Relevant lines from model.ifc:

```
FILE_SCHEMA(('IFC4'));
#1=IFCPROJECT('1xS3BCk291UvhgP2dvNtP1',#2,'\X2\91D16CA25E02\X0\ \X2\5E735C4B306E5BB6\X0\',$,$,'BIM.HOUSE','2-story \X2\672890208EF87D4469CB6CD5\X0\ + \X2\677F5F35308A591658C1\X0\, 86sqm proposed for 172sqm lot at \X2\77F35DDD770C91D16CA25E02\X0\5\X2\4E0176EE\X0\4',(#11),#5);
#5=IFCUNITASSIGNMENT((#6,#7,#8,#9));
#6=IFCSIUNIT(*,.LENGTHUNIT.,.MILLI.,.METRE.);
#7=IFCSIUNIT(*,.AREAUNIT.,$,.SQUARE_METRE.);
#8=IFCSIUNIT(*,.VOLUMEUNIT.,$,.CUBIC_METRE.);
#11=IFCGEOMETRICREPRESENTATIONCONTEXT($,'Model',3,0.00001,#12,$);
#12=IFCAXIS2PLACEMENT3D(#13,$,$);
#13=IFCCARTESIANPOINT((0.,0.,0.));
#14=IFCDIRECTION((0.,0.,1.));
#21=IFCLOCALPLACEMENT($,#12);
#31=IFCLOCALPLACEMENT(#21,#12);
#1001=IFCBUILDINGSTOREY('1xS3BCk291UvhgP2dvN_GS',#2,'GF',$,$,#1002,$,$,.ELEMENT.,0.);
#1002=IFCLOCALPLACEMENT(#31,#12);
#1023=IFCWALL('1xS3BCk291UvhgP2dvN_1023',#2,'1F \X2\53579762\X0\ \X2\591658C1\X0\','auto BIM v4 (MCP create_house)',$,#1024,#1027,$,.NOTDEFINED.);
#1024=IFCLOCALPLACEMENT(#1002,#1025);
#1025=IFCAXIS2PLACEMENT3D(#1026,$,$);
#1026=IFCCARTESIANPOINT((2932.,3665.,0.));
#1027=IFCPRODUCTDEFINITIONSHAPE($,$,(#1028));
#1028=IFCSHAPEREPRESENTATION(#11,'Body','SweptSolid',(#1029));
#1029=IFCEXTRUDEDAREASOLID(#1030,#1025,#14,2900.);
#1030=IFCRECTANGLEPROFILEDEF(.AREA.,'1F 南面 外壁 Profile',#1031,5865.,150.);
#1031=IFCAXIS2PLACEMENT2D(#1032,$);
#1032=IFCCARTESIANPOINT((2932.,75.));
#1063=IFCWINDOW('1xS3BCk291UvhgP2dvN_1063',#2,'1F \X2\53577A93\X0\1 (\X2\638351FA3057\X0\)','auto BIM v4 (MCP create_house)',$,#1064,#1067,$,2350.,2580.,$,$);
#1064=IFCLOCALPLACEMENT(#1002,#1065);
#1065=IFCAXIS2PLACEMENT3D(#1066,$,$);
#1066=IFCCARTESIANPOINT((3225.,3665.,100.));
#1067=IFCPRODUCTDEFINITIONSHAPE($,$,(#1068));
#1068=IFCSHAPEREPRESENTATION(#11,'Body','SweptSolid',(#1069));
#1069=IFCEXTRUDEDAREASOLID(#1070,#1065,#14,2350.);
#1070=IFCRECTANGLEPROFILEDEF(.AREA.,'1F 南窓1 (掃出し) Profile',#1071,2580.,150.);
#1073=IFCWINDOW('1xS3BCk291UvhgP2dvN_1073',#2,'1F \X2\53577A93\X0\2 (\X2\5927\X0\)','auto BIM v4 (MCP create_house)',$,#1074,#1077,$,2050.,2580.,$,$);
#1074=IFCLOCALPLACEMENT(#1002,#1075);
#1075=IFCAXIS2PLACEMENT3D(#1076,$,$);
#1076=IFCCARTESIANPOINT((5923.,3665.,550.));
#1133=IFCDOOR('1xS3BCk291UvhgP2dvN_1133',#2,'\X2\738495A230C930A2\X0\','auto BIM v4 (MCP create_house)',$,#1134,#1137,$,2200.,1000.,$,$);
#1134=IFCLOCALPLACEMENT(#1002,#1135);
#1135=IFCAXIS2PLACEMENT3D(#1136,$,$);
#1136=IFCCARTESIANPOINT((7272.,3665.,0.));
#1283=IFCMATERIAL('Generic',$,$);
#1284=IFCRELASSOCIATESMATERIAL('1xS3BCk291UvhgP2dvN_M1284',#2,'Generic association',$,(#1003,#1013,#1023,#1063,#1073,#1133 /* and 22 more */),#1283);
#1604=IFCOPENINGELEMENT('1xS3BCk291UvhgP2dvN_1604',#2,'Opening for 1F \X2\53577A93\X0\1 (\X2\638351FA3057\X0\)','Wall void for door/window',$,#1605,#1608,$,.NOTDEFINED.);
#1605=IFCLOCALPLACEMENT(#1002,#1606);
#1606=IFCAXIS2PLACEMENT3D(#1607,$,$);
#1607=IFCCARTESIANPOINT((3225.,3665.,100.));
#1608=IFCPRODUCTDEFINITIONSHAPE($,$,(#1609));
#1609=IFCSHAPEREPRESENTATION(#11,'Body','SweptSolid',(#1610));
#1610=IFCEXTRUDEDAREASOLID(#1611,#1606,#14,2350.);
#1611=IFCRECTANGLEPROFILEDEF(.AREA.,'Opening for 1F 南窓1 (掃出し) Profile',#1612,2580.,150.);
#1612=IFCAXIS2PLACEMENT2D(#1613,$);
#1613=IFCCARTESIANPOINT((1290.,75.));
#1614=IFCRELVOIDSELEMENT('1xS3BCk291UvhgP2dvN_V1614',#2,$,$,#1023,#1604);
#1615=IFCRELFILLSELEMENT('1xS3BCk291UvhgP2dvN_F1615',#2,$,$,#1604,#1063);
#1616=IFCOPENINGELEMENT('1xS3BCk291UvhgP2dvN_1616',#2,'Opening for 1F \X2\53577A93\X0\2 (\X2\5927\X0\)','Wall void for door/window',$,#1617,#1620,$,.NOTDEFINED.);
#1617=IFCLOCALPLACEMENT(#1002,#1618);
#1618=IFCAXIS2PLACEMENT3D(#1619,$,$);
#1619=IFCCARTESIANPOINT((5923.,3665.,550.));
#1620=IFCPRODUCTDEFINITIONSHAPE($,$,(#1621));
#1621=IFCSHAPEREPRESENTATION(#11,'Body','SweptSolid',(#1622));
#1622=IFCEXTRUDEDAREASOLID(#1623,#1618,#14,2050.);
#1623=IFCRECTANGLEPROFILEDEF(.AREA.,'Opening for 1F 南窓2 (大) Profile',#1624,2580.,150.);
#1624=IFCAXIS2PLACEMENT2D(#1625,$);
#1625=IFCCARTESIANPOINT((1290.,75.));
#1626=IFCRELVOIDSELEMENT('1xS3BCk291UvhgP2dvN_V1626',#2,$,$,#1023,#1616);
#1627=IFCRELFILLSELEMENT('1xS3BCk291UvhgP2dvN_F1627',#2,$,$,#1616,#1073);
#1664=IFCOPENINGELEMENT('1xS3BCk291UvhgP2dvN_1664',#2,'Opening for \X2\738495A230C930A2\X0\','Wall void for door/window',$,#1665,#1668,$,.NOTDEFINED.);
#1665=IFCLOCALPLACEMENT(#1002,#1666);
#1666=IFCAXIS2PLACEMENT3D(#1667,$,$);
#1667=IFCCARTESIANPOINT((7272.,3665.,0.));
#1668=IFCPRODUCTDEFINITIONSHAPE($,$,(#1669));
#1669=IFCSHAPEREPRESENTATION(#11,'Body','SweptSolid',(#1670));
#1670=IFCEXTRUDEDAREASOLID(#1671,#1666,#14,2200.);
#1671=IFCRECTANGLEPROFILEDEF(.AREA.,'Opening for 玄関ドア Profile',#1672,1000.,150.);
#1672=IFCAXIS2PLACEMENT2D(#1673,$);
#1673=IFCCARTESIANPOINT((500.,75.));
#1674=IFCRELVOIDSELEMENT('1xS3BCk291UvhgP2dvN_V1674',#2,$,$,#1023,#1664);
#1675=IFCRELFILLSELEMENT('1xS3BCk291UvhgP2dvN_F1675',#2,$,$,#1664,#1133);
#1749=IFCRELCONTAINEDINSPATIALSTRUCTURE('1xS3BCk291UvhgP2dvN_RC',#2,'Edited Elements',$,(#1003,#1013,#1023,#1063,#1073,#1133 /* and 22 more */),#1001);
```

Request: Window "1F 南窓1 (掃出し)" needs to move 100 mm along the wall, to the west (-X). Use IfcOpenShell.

```python
import ifcopenshell
import ifcopenshell.api.geometry
import ifcopenshell.util.placement
import ifcopenshell.util.unit

model = ifcopenshell.open("model.ifc")
unit_scale = ifcopenshell.util.unit.calculate_unit_scale(model)

window = model.by_guid("1xS3BCk291UvhgP2dvN_1063")
opening = window.FillsVoids[0].RelatingOpeningElement
wall = opening.VoidsElements[0].RelatingBuildingElement

wall_matrix = ifcopenshell.util.placement.get_local_placement(wall.ObjectPlacement)
shift = wall_matrix[:3, 0] * -0.1 / unit_scale
before = ifcopenshell.util.placement.get_local_placement(window.ObjectPlacement)[:3, 3].copy()

# The window is not placed relative to its opening, so move both.
for product in (opening, window):
    matrix = ifcopenshell.util.placement.get_local_placement(product.ObjectPlacement)
    matrix[:3, 3] += shift
    ifcopenshell.api.geometry.edit_object_placement(model, product=product, matrix=matrix, is_si=False)

after = ifcopenshell.util.placement.get_local_placement(window.ObjectPlacement)[:3, 3]
print("window moved by", (after - before).round(3) + 0.0)

model.write("model_v2.ifc")
```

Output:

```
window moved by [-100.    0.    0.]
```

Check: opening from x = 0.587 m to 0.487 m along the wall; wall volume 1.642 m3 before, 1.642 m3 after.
